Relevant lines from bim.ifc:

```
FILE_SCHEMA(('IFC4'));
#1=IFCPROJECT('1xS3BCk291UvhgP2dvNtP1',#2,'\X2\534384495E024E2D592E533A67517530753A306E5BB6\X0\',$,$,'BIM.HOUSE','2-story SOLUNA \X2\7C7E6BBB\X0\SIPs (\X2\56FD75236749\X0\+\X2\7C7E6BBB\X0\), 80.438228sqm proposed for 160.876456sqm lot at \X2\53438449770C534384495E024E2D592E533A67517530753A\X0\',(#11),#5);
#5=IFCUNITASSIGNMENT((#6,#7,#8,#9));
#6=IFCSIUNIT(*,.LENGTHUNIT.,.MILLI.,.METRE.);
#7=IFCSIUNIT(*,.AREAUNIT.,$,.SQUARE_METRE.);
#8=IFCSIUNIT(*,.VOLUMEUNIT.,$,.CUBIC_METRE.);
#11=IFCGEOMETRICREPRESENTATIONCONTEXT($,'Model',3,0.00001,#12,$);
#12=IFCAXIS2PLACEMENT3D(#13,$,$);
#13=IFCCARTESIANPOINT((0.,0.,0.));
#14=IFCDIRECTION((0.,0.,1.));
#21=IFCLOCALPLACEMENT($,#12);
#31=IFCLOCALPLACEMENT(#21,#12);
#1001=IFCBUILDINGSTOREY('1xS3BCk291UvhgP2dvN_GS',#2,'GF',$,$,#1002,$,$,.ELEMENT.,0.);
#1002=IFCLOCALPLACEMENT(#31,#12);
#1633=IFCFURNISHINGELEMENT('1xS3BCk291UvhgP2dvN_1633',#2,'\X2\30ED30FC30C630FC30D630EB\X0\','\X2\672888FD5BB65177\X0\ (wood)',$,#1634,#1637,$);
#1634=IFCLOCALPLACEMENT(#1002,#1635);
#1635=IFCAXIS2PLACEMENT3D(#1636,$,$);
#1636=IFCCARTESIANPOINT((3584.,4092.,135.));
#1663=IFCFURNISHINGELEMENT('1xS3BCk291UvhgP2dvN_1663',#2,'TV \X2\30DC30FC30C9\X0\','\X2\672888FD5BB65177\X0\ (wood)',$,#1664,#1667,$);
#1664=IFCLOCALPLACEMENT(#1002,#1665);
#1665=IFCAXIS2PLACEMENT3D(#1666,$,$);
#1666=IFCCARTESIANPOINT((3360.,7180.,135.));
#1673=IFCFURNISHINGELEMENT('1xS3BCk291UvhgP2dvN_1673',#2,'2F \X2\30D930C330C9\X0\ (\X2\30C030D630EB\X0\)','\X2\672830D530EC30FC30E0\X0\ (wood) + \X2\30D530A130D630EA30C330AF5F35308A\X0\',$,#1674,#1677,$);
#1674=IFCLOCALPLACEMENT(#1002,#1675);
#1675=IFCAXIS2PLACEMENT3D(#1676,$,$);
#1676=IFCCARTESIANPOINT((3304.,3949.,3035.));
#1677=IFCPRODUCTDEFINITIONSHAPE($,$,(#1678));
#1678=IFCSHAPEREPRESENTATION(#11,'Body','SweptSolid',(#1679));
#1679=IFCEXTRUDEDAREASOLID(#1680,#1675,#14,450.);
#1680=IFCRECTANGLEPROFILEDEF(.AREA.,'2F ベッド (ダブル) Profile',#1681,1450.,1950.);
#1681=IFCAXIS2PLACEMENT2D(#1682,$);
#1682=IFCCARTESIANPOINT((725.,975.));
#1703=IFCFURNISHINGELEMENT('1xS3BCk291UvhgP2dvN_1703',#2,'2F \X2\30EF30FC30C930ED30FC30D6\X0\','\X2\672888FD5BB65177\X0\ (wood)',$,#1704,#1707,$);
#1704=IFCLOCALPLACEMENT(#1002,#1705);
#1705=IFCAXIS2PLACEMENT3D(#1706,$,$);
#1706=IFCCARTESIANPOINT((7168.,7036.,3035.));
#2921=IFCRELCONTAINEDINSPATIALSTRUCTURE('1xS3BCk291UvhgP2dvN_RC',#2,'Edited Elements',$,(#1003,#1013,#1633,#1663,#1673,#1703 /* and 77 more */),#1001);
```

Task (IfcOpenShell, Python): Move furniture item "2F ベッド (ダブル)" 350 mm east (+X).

```python
import ifcopenshell
import ifcopenshell.api.geometry
import ifcopenshell.util.placement

model = ifcopenshell.open("bim.ifc")

item = model.by_guid("1xS3BCk291UvhgP2dvN_1673")
matrix = ifcopenshell.util.placement.get_local_placement(item.ObjectPlacement)
matrix[0, 3] += 350.0
ifcopenshell.api.geometry.edit_object_placement(model, product=item, matrix=matrix, is_si=False)

print(ifcopenshell.util.placement.get_local_placement(item.ObjectPlacement).round(3) + 0.0)

model.write("bim_edited.ifc")
```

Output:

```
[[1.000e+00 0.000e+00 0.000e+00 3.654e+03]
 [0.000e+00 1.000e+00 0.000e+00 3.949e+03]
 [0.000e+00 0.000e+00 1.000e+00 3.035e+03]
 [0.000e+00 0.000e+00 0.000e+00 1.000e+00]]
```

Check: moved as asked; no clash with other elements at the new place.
